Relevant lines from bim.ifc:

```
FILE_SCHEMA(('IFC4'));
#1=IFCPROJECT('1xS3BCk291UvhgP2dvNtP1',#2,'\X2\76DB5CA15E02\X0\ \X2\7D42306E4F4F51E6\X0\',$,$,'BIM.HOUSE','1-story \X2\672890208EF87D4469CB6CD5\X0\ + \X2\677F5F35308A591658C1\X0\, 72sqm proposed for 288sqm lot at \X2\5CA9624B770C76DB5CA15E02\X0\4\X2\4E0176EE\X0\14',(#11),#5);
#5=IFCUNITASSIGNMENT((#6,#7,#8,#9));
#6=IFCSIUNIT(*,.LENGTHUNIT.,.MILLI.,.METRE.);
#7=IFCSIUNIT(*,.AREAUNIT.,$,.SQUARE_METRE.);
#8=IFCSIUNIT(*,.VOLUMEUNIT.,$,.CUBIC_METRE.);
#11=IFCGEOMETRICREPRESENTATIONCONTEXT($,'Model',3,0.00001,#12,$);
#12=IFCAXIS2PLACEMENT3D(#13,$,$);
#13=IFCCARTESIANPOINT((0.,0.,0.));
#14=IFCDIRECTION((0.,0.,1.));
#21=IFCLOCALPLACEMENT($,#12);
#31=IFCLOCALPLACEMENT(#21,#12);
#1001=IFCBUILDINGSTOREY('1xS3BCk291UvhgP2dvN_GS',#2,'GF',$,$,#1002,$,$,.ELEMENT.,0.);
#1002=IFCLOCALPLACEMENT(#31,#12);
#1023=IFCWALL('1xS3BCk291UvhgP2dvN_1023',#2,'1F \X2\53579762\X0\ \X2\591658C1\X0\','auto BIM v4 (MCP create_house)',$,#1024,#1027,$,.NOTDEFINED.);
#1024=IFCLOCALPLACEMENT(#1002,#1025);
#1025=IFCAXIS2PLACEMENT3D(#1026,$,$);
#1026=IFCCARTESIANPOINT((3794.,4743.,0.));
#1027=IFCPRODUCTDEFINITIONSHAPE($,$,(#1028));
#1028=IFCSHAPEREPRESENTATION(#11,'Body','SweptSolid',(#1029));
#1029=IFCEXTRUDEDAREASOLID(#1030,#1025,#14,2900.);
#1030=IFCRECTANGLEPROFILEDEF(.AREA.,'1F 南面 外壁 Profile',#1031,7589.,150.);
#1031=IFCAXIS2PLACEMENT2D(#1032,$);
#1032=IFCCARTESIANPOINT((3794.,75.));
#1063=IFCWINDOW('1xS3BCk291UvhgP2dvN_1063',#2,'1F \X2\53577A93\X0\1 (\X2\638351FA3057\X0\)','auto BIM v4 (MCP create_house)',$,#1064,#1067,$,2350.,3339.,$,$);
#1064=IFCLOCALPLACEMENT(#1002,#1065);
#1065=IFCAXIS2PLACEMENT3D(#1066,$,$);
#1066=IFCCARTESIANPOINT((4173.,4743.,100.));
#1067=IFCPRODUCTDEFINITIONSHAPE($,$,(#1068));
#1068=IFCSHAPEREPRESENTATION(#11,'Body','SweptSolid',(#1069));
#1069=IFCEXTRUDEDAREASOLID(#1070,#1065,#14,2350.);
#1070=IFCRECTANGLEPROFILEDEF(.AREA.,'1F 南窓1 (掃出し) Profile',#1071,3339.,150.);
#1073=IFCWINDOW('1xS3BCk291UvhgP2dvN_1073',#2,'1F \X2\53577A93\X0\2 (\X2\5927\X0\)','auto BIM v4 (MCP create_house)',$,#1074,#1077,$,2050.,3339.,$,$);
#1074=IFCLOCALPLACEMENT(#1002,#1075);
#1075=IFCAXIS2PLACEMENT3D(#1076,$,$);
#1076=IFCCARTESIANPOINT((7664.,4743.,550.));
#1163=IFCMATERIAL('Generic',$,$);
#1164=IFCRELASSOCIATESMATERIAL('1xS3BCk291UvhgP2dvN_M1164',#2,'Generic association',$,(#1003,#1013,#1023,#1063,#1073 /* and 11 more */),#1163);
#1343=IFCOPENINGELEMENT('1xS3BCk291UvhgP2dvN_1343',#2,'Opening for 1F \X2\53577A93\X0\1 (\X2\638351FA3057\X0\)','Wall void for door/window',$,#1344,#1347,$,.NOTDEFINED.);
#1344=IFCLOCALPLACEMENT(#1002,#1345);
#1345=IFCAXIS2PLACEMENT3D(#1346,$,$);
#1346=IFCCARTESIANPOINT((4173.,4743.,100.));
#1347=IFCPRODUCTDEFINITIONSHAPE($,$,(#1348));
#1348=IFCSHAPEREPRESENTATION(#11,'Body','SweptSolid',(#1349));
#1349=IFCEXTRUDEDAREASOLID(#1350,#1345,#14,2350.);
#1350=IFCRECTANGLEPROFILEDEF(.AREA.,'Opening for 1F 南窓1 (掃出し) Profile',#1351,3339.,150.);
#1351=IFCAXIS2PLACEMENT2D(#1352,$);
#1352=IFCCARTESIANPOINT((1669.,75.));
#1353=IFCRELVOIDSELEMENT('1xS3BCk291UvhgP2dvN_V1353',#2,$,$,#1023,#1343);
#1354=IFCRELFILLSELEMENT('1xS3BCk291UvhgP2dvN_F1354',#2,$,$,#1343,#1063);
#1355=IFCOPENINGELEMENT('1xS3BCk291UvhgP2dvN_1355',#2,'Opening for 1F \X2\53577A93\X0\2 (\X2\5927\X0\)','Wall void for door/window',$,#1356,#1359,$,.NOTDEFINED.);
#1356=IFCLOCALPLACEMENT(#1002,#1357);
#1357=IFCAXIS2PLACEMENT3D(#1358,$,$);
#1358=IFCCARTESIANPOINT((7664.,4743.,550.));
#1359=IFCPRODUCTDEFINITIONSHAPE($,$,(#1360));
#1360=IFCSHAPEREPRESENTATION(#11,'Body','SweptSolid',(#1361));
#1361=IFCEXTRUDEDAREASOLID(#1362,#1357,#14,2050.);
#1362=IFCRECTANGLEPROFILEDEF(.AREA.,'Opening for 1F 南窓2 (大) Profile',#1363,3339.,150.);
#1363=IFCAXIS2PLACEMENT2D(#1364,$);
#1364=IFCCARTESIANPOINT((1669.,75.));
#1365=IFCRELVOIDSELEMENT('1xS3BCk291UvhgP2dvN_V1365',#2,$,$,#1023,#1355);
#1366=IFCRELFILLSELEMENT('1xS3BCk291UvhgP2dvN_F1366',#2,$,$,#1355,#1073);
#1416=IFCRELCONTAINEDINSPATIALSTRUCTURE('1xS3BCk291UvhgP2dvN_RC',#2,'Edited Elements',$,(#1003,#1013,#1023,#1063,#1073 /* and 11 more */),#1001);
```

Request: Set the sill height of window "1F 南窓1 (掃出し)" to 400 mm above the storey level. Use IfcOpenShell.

```python
import numpy as np
import ifcopenshell
import ifcopenshell.api.geometry
import ifcopenshell.geom
import ifcopenshell.util.element
import ifcopenshell.util.placement
import ifcopenshell.util.shape
import ifcopenshell.util.unit

model = ifcopenshell.open("bim.ifc")
unit_scale = ifcopenshell.util.unit.calculate_unit_scale(model)

window = model.by_guid("1xS3BCk291UvhgP2dvN_1063")
opening = window.FillsVoids[0].RelatingOpeningElement
storey = ifcopenshell.util.element.get_container(window, ifc_class="IfcBuildingStorey")
level = ifcopenshell.util.placement.get_local_placement(storey.ObjectPlacement)[2, 3]

# The opening's origin need not be at the sill, so measure its lowest point.
shape = ifcopenshell.geom.create_shape(ifcopenshell.geom.settings(), opening)
bottom = ifcopenshell.util.shape.get_shape_bottom_elevation(shape, shape.geometry) / unit_scale
dz = level + 0.4 / unit_scale - bottom

shift = np.array([0.0, 0.0, dz])
# The window is not placed relative to its opening, so move both.
for product in (opening, window):
    matrix = ifcopenshell.util.placement.get_local_placement(product.ObjectPlacement)
    matrix[:3, 3] += shift
    ifcopenshell.api.geometry.edit_object_placement(model, product=product, matrix=matrix, is_si=False)

print(f"moved by {dz * unit_scale:+.3f} m")

model.write("bim_updated.ifc")
```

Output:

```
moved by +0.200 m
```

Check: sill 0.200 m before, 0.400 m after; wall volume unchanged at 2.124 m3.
